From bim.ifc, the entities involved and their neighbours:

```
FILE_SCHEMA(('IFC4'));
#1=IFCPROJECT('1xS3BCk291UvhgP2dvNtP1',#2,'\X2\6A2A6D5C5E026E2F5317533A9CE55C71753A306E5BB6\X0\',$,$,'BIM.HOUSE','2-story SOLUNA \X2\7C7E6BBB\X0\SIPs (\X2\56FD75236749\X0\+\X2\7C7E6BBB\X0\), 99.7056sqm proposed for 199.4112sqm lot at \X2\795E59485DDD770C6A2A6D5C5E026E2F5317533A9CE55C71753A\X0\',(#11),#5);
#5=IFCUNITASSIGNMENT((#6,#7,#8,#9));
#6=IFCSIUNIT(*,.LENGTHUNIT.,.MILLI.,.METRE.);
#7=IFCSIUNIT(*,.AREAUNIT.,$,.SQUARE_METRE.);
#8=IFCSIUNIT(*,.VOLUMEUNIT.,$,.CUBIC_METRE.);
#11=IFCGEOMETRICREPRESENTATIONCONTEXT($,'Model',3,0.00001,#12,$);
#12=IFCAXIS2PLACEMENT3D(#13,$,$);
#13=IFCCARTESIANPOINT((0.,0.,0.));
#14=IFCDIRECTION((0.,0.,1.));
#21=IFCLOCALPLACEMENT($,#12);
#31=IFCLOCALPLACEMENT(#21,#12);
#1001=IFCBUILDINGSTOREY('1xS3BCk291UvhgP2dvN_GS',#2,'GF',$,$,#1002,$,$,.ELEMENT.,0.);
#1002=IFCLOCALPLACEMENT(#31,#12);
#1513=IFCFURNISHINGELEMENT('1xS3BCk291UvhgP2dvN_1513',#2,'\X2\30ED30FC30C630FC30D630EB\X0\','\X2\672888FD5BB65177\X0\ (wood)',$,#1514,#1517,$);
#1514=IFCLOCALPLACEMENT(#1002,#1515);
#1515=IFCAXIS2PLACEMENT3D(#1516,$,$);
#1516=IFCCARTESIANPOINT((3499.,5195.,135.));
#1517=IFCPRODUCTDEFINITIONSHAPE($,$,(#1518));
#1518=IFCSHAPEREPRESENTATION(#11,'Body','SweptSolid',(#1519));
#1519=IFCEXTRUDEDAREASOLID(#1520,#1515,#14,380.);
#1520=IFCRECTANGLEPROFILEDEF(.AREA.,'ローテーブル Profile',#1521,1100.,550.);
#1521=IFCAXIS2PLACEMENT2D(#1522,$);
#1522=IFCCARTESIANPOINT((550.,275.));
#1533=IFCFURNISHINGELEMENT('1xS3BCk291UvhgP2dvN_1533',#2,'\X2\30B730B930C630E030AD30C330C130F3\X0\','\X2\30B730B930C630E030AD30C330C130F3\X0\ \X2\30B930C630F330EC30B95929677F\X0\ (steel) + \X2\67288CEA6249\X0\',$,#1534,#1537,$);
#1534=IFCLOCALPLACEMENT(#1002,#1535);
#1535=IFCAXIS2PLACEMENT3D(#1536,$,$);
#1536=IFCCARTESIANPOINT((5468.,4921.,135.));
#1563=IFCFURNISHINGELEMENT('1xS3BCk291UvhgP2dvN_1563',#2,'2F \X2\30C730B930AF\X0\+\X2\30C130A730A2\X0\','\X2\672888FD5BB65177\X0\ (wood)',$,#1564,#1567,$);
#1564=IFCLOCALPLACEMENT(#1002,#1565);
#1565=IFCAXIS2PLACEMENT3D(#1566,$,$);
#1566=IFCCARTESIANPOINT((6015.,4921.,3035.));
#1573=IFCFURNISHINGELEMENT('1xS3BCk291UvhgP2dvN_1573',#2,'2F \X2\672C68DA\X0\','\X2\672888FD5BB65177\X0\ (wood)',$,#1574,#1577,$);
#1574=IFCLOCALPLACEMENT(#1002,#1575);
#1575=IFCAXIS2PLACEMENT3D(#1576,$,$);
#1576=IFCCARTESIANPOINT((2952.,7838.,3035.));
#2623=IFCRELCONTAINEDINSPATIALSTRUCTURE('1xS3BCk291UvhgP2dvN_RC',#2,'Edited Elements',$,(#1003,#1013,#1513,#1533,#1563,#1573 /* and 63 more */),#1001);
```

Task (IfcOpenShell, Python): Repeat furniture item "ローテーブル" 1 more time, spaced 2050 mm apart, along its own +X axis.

```python
import ifcopenshell
import ifcopenshell.api.geometry
import ifcopenshell.api.root
import ifcopenshell.util.element
import ifcopenshell.util.placement
import ifcopenshell.util.unit

model = ifcopenshell.open("bim.ifc")
unit_scale = ifcopenshell.util.unit.calculate_unit_scale(model)


def reuse_history(source, copy):
    """copy_class also copies each property set's owner history, people and application; keep the originals."""
    for rel in copy.IsDefinedBy:
        if rel.is_a("IfcRelDefinesByProperties") and (history := rel.RelatingPropertyDefinition.OwnerHistory):
            rel.RelatingPropertyDefinition.OwnerHistory = source.OwnerHistory
            ifcopenshell.util.element.remove_deep2(model, history)


source = model.by_id(1513)
base = ifcopenshell.util.placement.get_local_placement(source.ObjectPlacement)
step = base[:3, 0] * 2.05 / unit_scale

for i in range(1, 2):
    copy = ifcopenshell.api.root.copy_class(model, product=source)
    copy.Representation = ifcopenshell.util.element.copy_deep(
        model, source.Representation, exclude=["IfcGeometricRepresentationContext", "IfcRepresentationMap"]
    )
    reuse_history(source, copy)
    matrix = base.copy()
    matrix[:3, 3] += i * step
    print("added at", matrix[:3, 3].round(3) + 0.0)
    ifcopenshell.api.geometry.edit_object_placement(model, product=copy, matrix=matrix, is_si=False)

model.write("bim_updated.ifc")
```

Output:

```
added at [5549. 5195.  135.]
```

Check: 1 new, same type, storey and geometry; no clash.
